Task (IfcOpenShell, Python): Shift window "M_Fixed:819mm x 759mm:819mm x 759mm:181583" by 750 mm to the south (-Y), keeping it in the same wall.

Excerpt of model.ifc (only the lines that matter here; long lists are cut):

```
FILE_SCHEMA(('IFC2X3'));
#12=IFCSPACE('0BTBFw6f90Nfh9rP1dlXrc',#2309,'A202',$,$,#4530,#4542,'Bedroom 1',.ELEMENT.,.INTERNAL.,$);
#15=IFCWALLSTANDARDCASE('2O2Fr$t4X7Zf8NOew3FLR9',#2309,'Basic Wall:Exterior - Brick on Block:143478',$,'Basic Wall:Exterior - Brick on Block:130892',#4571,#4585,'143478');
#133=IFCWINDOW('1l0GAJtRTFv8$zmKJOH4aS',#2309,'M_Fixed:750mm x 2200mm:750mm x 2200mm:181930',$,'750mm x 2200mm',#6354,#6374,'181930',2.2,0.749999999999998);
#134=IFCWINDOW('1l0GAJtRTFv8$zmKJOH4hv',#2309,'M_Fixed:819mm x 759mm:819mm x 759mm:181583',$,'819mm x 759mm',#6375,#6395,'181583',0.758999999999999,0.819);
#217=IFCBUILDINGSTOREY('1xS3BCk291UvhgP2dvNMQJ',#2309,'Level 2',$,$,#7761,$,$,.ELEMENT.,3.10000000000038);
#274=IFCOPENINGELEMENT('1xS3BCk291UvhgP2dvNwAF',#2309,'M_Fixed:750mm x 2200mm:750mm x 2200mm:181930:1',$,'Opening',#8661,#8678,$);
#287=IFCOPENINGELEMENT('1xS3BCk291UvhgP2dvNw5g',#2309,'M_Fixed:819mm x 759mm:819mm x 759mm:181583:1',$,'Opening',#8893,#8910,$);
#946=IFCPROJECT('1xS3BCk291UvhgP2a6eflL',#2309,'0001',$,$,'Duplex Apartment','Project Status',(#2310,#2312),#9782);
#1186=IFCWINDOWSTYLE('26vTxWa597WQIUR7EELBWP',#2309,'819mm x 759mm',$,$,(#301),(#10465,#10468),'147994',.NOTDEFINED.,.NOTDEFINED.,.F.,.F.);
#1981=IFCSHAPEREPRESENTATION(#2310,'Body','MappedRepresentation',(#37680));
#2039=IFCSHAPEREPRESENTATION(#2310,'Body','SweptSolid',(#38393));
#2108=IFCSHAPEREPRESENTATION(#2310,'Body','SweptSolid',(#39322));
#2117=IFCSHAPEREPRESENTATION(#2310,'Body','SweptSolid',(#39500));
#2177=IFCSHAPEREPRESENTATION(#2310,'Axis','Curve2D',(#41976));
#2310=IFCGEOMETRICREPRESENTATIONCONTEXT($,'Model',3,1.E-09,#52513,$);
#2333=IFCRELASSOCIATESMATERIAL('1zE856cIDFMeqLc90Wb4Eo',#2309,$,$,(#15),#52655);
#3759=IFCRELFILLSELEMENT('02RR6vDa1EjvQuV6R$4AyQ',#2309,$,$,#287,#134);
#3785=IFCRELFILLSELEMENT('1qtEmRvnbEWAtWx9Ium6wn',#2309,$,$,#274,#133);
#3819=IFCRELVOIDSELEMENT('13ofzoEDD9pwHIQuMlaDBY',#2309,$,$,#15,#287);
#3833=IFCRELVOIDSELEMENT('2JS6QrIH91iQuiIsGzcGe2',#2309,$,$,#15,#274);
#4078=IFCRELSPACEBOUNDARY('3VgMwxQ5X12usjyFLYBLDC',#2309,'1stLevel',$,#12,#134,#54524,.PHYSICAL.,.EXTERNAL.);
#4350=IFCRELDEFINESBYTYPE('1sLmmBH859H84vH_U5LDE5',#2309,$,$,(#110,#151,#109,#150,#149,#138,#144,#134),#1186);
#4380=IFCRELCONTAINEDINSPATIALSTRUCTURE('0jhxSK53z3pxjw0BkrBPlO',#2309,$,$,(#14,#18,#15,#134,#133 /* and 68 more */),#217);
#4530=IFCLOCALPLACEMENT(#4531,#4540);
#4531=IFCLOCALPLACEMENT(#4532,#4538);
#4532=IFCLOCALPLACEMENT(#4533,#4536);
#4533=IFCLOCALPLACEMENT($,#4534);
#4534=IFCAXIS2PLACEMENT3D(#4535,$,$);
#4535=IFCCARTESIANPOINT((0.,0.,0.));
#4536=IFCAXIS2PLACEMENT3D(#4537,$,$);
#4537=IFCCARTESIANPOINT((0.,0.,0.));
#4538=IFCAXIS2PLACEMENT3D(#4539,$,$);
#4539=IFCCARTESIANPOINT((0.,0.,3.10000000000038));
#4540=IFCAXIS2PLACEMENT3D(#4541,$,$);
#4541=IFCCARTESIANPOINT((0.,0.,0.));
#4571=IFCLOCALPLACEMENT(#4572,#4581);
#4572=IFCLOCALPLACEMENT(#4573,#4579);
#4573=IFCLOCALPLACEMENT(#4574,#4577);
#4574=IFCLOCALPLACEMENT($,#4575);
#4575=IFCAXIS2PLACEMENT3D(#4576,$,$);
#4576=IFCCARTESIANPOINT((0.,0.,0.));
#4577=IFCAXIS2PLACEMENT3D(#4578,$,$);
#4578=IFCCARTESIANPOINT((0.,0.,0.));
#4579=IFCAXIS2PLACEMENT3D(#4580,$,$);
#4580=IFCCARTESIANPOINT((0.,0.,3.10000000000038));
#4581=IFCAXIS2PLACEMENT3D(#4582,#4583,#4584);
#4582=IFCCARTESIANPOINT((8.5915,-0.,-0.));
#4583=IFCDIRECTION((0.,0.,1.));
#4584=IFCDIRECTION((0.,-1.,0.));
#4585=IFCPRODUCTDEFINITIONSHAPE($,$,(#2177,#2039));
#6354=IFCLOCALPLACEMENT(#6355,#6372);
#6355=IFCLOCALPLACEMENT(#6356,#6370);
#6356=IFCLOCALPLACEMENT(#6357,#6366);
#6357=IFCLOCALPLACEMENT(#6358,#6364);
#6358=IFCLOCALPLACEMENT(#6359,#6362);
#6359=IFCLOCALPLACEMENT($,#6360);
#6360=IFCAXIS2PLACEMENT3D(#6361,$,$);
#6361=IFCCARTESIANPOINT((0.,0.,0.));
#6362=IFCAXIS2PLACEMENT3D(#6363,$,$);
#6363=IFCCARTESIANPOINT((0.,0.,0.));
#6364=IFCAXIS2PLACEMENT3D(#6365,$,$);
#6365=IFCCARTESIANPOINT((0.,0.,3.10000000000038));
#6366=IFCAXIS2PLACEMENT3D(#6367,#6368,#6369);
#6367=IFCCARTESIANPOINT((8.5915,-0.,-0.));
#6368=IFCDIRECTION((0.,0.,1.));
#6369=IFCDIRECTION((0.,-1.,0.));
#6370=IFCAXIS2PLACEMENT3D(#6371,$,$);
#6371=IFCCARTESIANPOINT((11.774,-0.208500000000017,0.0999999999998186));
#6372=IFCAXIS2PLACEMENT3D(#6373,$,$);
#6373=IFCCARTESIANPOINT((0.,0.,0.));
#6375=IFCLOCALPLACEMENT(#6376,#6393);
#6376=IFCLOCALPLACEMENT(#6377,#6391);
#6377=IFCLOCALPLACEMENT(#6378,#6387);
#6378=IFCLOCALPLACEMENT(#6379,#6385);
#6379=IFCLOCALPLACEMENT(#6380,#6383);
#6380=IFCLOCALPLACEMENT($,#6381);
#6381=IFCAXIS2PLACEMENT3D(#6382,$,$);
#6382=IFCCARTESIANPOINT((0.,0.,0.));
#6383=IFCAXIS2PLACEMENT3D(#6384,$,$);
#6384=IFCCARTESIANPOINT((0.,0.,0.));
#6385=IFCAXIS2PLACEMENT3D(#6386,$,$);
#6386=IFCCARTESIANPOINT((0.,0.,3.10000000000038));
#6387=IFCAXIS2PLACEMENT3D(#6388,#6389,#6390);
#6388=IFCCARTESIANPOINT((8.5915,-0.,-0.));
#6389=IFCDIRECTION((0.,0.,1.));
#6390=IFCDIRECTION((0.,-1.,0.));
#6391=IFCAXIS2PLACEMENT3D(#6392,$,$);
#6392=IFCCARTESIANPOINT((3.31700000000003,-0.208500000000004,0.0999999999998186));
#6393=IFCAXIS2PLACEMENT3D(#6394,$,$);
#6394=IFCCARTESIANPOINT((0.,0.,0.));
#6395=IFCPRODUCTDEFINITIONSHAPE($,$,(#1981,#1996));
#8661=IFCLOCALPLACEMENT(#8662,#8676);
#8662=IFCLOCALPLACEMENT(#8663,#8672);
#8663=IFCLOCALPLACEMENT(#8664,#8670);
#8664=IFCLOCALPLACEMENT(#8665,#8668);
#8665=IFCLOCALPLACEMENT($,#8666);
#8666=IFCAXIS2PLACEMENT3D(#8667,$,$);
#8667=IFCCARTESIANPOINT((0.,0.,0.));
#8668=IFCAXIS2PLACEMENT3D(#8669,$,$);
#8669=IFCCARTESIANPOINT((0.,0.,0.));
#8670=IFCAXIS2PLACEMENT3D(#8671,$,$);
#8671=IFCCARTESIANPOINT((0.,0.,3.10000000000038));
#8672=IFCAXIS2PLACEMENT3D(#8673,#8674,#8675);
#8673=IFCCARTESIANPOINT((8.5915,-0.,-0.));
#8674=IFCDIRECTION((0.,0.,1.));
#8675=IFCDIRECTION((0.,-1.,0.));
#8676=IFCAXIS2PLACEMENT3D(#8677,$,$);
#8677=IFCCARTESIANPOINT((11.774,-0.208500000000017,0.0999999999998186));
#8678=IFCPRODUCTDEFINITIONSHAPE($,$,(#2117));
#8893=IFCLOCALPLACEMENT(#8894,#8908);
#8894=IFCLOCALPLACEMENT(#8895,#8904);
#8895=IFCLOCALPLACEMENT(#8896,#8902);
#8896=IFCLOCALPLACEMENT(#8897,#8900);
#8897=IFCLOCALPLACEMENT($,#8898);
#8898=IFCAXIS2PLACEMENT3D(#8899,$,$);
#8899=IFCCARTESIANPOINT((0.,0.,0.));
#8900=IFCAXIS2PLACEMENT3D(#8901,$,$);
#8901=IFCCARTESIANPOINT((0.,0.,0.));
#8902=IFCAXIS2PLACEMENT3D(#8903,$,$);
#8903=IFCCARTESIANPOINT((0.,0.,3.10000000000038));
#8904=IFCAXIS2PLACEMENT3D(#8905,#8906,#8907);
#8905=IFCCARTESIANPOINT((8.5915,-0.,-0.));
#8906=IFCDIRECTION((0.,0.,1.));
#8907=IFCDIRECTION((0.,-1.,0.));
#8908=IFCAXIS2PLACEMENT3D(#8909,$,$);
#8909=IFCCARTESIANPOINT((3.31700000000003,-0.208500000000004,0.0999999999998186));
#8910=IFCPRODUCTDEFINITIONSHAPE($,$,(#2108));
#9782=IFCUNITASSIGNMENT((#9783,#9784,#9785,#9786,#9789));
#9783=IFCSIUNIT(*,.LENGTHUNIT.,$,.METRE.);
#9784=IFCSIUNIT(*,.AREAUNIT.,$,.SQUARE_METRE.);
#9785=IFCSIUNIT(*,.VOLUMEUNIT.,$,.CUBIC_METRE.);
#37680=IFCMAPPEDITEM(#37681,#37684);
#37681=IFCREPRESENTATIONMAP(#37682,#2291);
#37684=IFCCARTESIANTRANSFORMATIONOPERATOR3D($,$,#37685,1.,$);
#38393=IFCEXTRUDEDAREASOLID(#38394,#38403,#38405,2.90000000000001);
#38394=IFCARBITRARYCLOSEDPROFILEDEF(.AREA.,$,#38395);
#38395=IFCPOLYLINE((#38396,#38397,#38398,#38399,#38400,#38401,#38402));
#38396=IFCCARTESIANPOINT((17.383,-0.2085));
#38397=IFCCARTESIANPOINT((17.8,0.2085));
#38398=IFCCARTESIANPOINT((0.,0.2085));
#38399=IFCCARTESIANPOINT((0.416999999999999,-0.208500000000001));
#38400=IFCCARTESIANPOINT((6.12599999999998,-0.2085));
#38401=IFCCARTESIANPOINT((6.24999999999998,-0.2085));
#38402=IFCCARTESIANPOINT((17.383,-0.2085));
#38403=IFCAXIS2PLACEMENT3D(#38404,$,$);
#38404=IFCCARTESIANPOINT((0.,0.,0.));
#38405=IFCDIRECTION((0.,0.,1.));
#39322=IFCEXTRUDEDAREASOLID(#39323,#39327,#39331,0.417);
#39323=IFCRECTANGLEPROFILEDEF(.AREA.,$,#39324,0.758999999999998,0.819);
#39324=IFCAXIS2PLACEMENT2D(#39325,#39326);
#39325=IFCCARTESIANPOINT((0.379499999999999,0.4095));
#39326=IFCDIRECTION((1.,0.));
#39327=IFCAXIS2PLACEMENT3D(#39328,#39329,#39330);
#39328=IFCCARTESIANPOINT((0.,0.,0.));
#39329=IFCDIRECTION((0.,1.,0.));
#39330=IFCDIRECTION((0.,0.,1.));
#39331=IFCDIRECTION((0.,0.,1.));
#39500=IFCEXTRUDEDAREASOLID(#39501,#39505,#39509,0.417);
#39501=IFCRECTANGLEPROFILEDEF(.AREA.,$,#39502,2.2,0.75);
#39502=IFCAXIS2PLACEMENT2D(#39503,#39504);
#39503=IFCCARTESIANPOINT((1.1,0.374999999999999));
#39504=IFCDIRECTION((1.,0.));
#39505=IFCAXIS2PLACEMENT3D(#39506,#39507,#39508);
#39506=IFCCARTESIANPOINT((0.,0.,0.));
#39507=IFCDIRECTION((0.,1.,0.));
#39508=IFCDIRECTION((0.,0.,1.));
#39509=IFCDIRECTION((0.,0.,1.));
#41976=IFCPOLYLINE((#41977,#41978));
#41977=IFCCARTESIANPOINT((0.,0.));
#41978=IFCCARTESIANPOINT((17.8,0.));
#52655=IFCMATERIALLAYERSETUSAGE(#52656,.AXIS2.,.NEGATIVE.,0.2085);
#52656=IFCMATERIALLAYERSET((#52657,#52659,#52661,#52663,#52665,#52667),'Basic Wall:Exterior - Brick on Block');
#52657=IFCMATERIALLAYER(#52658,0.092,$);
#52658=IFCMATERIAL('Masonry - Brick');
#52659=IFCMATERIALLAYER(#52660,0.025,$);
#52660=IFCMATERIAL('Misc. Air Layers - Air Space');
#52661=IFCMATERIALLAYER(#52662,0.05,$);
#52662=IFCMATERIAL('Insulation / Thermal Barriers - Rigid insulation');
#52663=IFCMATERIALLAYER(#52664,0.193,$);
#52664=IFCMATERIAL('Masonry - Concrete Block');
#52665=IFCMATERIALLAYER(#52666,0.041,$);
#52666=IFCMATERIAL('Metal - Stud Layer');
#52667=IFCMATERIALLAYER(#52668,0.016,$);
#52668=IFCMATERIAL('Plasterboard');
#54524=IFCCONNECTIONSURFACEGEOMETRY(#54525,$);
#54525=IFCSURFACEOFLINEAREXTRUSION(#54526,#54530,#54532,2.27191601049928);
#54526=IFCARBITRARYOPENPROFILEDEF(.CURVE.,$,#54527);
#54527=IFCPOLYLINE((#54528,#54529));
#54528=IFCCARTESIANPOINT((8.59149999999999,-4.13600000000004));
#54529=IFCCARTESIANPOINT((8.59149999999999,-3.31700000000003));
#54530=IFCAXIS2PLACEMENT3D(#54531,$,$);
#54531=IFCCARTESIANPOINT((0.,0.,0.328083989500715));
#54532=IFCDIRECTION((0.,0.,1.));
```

```python
import numpy as np
import ifcopenshell
import ifcopenshell.api.geometry
import ifcopenshell.util.placement
import ifcopenshell.util.unit

model = ifcopenshell.open("model.ifc")
unit_scale = ifcopenshell.util.unit.calculate_unit_scale(model)

window = model.by_guid("1l0GAJtRTFv8$zmKJOH4hv")
opening = window.FillsVoids[0].RelatingOpeningElement
wall = opening.VoidsElements[0].RelatingBuildingElement

wall_matrix = ifcopenshell.util.placement.get_local_placement(wall.ObjectPlacement)
shift = wall_matrix[:3, 0] * 0.75 / unit_scale
before = ifcopenshell.util.placement.get_local_placement(window.ObjectPlacement)[:3, 3].copy()

# The window is not placed relative to its opening, so move both.
for product in (opening, window):
    matrix = ifcopenshell.util.placement.get_local_placement(product.ObjectPlacement)
    matrix[:3, 3] += shift
    ifcopenshell.api.geometry.edit_object_placement(model, product=product, matrix=matrix, is_si=False)

# Space boundary surfaces are stored in each space's coordinates; move them too.
for rel in window.ProvidesBoundaries:
    if not rel.ConnectionGeometry:
        continue
    surface = rel.ConnectionGeometry.SurfaceOnRelatingElement
    space_matrix = ifcopenshell.util.placement.get_local_placement(rel.RelatingSpace.ObjectPlacement)
    point = np.array(surface.Position.Location.Coordinates) + space_matrix[:3, :3].T @ shift
    surface.Position = model.createIfcAxis2Placement3D(
        model.createIfcCartesianPoint(point.tolist()), surface.Position.Axis, surface.Position.RefDirection
    )

after = ifcopenshell.util.placement.get_local_placement(window.ObjectPlacement)[:3, 3]
print("window moved by", (after - before).round(3) + 0.0)

model.write("model_updated.ifc")
```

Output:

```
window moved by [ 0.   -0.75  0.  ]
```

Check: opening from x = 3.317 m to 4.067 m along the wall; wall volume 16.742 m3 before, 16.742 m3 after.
